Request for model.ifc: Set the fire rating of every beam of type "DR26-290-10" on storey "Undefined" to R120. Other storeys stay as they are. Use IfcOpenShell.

First a look at what the model holds.

```python
import ifcopenshell
import ifcopenshell.util.element

model = ifcopenshell.open("model.ifc")
print(model.schema)
storey = next(s for s in model.by_type("IfcBuildingStorey") if s.Name == "Undefined")
beams = [e for e in ifcopenshell.util.element.get_decomposition(storey) if e.is_a("IfcBeam")]
seen = {}
for e in beams:
    element_type = ifcopenshell.util.element.get_type(e)
    key = (element_type.Name if element_type != e and element_type else None, ifcopenshell.util.element.get_pset(e, "Pset_BeamCommon", "FireRating"))
    seen[key] = seen.get(key, 0) + 1
for (name, value), count in sorted(seen.items(), key=str):
    print(count, "x", name, "|", value)
```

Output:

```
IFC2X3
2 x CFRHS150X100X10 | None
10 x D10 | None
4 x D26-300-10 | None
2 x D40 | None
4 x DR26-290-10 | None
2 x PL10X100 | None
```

```python
import ifcopenshell
import ifcopenshell.api.pset
import ifcopenshell.util.element

model = ifcopenshell.open("model.ifc")

storey = next(s for s in model.by_type("IfcBuildingStorey") if s.Name == "Undefined")
beams = [e for e in ifcopenshell.util.element.get_decomposition(storey) if e.is_a("IfcBeam")]

count = 0
for e in beams:
    element_type = ifcopenshell.util.element.get_type(e)
    if element_type in (None, e) or element_type.Name != "DR26-290-10":
        continue
    found = ifcopenshell.util.element.get_pset(e, "Pset_BeamCommon", should_inherit=False)
    if found:
        pset = model.by_id(found["id"])
        if len(ifcopenshell.util.element.get_elements_by_pset(pset)) > 1:
            pset = ifcopenshell.api.pset.unshare_pset(model, products=[e], pset=pset)[0]
    else:
        pset = ifcopenshell.api.pset.add_pset(model, product=e, name="Pset_BeamCommon")
    ifcopenshell.api.pset.edit_pset(model, pset=pset, properties={"FireRating": "R120"})
    count += 1

print(count, "beams updated")

model.write("model-out.ifc")
```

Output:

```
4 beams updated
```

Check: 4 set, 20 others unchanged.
